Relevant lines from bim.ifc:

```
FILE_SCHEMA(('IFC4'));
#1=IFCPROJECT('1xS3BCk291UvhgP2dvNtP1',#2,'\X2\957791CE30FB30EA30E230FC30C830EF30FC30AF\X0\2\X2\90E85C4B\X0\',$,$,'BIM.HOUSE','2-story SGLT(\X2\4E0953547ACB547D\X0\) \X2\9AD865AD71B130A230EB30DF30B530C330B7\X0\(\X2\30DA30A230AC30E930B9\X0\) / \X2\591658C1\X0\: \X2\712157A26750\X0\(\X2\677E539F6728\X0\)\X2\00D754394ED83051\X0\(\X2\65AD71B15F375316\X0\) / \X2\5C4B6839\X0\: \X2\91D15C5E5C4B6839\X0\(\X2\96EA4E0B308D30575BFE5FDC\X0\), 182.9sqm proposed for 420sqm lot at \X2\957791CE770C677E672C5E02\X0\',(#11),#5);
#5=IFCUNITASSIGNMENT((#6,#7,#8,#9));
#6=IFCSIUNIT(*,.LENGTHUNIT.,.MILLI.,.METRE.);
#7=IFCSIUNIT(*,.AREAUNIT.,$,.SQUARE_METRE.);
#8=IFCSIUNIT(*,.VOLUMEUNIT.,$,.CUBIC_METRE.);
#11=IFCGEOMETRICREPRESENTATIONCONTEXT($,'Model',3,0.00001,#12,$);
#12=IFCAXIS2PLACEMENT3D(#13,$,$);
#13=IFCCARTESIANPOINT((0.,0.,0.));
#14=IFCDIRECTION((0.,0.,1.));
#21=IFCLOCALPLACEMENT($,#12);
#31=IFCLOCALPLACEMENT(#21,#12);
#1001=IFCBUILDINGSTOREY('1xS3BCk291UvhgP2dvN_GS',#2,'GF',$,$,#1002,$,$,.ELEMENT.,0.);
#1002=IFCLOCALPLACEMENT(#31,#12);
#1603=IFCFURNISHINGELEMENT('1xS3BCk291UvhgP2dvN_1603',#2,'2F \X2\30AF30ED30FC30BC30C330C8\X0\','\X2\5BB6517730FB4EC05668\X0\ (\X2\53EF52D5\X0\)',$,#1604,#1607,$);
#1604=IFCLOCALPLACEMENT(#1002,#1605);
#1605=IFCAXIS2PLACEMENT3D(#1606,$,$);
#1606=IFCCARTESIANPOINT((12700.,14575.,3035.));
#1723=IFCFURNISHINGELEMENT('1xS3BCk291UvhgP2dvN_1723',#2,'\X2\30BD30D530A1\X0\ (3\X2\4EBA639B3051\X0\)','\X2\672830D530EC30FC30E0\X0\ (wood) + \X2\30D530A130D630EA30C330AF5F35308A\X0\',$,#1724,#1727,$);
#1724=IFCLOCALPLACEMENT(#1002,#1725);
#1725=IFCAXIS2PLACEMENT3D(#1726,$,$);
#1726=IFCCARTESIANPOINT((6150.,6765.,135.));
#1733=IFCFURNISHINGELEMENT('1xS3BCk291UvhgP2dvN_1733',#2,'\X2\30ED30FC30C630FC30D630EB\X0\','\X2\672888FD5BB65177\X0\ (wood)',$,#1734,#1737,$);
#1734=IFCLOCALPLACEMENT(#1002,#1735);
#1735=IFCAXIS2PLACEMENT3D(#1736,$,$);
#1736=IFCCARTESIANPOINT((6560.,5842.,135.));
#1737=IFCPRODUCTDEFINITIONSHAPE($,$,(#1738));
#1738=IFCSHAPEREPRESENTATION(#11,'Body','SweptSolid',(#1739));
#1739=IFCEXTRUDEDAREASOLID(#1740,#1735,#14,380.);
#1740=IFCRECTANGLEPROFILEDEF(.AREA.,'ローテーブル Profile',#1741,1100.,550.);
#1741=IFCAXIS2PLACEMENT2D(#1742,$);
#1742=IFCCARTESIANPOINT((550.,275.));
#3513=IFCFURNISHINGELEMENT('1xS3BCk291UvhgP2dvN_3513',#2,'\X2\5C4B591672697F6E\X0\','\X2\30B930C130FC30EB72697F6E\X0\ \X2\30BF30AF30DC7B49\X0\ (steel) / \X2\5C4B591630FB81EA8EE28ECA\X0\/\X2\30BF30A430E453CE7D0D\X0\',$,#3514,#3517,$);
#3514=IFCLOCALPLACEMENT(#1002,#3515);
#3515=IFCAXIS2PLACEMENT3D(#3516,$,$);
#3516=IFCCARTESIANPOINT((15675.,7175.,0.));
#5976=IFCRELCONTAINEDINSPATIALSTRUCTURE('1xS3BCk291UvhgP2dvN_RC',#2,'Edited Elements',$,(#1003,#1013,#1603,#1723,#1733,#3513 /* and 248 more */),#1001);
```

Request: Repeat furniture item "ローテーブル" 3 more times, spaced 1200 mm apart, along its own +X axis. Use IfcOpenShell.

```python
import ifcopenshell
import ifcopenshell.api.geometry
import ifcopenshell.api.root
import ifcopenshell.util.element
import ifcopenshell.util.placement

model = ifcopenshell.open("bim.ifc")


def reuse_history(source, copy):
    """copy_class also copies each property set's owner history, people and application; keep the originals."""
    for rel in copy.IsDefinedBy:
        if rel.is_a("IfcRelDefinesByProperties") and (history := rel.RelatingPropertyDefinition.OwnerHistory):
            rel.RelatingPropertyDefinition.OwnerHistory = source.OwnerHistory
            ifcopenshell.util.element.remove_deep2(model, history)


source = model.by_guid("1xS3BCk291UvhgP2dvN_1733")
base = ifcopenshell.util.placement.get_local_placement(source.ObjectPlacement)
step = base[:3, 0] * 1200.0

for i in range(1, 4):
    copy = ifcopenshell.api.root.copy_class(model, product=source)
    copy.Representation = ifcopenshell.util.element.copy_deep(
        model, source.Representation, exclude=["IfcGeometricRepresentationContext", "IfcRepresentationMap"]
    )
    reuse_history(source, copy)
    matrix = base.copy()
    matrix[:3, 3] += i * step
    print("added at", matrix[:3, 3].round(3) + 0.0)
    ifcopenshell.api.geometry.edit_object_placement(model, product=copy, matrix=matrix, is_si=False)

model.write("bim-out.ifc")
```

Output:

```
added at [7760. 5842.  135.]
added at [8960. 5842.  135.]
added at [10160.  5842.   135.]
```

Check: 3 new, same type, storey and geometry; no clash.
